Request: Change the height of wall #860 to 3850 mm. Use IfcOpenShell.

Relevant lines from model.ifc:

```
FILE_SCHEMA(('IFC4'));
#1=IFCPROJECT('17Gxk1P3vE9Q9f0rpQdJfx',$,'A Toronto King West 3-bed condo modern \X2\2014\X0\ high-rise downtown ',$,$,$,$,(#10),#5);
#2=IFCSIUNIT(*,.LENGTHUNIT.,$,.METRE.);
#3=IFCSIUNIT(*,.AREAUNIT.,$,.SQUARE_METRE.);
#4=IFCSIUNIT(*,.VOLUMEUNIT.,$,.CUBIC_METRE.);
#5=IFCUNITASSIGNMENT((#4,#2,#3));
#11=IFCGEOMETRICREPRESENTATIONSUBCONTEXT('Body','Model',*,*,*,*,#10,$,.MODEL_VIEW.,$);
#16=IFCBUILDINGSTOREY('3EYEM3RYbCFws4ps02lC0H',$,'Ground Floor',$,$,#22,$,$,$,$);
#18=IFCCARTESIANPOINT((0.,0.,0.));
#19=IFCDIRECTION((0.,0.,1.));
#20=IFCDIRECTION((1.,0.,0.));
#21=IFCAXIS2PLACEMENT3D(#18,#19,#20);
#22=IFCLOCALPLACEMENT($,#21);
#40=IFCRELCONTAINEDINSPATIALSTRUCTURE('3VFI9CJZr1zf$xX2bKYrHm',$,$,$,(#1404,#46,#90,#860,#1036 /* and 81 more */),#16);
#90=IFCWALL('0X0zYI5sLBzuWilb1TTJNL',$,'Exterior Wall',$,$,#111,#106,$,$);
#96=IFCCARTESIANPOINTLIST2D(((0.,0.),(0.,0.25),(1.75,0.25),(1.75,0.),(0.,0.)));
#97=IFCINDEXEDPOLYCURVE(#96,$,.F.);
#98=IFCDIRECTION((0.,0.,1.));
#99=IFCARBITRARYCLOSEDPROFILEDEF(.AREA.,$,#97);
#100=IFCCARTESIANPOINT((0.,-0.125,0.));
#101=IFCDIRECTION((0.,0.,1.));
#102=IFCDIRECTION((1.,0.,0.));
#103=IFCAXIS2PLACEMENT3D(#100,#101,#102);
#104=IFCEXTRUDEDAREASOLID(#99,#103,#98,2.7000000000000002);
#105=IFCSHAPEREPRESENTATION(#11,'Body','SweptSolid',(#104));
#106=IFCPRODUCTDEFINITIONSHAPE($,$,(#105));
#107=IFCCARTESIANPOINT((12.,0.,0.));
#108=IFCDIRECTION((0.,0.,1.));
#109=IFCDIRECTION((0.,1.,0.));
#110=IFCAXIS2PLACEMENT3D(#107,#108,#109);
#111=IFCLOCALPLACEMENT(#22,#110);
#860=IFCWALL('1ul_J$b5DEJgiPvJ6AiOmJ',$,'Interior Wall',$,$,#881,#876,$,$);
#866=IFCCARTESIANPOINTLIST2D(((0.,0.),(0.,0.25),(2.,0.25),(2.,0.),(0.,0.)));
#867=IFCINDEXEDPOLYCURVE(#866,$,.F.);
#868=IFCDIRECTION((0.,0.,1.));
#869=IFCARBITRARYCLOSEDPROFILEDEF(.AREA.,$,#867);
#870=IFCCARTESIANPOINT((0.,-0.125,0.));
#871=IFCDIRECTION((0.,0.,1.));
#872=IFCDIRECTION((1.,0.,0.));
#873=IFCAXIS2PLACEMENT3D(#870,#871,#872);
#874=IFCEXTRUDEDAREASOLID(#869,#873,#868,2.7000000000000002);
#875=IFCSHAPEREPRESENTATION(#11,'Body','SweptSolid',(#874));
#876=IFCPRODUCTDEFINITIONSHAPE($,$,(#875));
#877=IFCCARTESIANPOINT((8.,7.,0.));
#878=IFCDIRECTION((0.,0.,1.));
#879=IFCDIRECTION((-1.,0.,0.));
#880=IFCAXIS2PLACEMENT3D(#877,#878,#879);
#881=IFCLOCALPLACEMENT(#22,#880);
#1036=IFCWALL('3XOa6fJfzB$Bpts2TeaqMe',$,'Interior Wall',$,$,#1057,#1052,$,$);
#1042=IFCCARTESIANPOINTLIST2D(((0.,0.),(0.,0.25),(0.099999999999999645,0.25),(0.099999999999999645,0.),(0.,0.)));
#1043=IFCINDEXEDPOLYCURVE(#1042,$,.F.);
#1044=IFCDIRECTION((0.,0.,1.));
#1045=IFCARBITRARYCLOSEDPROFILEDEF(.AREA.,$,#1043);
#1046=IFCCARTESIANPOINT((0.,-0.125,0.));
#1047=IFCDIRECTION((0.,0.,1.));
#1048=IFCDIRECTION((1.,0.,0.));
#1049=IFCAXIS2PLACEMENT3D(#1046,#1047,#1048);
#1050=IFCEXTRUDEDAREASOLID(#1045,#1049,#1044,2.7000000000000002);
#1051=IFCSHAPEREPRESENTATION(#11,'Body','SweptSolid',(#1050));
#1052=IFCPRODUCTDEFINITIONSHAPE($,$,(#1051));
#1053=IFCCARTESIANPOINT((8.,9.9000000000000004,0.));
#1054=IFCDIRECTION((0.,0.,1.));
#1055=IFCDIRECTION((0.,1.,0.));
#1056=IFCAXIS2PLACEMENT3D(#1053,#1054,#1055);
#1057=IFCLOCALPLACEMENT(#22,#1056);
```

```python
import ifcopenshell
import ifcopenshell.geom
import ifcopenshell.util.representation
import ifcopenshell.util.shape
import ifcopenshell.util.unit

model = ifcopenshell.open("model.ifc")
unit_scale = ifcopenshell.util.unit.calculate_unit_scale(model)
settings = ifcopenshell.geom.settings()


def volume(element):
    """Net volume in cubic metres, openings subtracted."""
    shape = ifcopenshell.geom.create_shape(settings, element)
    return ifcopenshell.util.shape.get_volume(shape.geometry)


wall = model.by_guid("1ul_J$b5DEJgiPvJ6AiOmJ")
before = volume(wall)

body = ifcopenshell.util.representation.get_representation(wall, "Model", "Body")
solid = body.Items[0]
old_height = solid.Depth
solid.Depth = 3.85 / unit_scale
after = volume(wall)

print(f"height {old_height:g} -> {solid.Depth:g}, volume {before:.3f} -> {after:.3f} m3")

model.write("model_edited.ifc")
```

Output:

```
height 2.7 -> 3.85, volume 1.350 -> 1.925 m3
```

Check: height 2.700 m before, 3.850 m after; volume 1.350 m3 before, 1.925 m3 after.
